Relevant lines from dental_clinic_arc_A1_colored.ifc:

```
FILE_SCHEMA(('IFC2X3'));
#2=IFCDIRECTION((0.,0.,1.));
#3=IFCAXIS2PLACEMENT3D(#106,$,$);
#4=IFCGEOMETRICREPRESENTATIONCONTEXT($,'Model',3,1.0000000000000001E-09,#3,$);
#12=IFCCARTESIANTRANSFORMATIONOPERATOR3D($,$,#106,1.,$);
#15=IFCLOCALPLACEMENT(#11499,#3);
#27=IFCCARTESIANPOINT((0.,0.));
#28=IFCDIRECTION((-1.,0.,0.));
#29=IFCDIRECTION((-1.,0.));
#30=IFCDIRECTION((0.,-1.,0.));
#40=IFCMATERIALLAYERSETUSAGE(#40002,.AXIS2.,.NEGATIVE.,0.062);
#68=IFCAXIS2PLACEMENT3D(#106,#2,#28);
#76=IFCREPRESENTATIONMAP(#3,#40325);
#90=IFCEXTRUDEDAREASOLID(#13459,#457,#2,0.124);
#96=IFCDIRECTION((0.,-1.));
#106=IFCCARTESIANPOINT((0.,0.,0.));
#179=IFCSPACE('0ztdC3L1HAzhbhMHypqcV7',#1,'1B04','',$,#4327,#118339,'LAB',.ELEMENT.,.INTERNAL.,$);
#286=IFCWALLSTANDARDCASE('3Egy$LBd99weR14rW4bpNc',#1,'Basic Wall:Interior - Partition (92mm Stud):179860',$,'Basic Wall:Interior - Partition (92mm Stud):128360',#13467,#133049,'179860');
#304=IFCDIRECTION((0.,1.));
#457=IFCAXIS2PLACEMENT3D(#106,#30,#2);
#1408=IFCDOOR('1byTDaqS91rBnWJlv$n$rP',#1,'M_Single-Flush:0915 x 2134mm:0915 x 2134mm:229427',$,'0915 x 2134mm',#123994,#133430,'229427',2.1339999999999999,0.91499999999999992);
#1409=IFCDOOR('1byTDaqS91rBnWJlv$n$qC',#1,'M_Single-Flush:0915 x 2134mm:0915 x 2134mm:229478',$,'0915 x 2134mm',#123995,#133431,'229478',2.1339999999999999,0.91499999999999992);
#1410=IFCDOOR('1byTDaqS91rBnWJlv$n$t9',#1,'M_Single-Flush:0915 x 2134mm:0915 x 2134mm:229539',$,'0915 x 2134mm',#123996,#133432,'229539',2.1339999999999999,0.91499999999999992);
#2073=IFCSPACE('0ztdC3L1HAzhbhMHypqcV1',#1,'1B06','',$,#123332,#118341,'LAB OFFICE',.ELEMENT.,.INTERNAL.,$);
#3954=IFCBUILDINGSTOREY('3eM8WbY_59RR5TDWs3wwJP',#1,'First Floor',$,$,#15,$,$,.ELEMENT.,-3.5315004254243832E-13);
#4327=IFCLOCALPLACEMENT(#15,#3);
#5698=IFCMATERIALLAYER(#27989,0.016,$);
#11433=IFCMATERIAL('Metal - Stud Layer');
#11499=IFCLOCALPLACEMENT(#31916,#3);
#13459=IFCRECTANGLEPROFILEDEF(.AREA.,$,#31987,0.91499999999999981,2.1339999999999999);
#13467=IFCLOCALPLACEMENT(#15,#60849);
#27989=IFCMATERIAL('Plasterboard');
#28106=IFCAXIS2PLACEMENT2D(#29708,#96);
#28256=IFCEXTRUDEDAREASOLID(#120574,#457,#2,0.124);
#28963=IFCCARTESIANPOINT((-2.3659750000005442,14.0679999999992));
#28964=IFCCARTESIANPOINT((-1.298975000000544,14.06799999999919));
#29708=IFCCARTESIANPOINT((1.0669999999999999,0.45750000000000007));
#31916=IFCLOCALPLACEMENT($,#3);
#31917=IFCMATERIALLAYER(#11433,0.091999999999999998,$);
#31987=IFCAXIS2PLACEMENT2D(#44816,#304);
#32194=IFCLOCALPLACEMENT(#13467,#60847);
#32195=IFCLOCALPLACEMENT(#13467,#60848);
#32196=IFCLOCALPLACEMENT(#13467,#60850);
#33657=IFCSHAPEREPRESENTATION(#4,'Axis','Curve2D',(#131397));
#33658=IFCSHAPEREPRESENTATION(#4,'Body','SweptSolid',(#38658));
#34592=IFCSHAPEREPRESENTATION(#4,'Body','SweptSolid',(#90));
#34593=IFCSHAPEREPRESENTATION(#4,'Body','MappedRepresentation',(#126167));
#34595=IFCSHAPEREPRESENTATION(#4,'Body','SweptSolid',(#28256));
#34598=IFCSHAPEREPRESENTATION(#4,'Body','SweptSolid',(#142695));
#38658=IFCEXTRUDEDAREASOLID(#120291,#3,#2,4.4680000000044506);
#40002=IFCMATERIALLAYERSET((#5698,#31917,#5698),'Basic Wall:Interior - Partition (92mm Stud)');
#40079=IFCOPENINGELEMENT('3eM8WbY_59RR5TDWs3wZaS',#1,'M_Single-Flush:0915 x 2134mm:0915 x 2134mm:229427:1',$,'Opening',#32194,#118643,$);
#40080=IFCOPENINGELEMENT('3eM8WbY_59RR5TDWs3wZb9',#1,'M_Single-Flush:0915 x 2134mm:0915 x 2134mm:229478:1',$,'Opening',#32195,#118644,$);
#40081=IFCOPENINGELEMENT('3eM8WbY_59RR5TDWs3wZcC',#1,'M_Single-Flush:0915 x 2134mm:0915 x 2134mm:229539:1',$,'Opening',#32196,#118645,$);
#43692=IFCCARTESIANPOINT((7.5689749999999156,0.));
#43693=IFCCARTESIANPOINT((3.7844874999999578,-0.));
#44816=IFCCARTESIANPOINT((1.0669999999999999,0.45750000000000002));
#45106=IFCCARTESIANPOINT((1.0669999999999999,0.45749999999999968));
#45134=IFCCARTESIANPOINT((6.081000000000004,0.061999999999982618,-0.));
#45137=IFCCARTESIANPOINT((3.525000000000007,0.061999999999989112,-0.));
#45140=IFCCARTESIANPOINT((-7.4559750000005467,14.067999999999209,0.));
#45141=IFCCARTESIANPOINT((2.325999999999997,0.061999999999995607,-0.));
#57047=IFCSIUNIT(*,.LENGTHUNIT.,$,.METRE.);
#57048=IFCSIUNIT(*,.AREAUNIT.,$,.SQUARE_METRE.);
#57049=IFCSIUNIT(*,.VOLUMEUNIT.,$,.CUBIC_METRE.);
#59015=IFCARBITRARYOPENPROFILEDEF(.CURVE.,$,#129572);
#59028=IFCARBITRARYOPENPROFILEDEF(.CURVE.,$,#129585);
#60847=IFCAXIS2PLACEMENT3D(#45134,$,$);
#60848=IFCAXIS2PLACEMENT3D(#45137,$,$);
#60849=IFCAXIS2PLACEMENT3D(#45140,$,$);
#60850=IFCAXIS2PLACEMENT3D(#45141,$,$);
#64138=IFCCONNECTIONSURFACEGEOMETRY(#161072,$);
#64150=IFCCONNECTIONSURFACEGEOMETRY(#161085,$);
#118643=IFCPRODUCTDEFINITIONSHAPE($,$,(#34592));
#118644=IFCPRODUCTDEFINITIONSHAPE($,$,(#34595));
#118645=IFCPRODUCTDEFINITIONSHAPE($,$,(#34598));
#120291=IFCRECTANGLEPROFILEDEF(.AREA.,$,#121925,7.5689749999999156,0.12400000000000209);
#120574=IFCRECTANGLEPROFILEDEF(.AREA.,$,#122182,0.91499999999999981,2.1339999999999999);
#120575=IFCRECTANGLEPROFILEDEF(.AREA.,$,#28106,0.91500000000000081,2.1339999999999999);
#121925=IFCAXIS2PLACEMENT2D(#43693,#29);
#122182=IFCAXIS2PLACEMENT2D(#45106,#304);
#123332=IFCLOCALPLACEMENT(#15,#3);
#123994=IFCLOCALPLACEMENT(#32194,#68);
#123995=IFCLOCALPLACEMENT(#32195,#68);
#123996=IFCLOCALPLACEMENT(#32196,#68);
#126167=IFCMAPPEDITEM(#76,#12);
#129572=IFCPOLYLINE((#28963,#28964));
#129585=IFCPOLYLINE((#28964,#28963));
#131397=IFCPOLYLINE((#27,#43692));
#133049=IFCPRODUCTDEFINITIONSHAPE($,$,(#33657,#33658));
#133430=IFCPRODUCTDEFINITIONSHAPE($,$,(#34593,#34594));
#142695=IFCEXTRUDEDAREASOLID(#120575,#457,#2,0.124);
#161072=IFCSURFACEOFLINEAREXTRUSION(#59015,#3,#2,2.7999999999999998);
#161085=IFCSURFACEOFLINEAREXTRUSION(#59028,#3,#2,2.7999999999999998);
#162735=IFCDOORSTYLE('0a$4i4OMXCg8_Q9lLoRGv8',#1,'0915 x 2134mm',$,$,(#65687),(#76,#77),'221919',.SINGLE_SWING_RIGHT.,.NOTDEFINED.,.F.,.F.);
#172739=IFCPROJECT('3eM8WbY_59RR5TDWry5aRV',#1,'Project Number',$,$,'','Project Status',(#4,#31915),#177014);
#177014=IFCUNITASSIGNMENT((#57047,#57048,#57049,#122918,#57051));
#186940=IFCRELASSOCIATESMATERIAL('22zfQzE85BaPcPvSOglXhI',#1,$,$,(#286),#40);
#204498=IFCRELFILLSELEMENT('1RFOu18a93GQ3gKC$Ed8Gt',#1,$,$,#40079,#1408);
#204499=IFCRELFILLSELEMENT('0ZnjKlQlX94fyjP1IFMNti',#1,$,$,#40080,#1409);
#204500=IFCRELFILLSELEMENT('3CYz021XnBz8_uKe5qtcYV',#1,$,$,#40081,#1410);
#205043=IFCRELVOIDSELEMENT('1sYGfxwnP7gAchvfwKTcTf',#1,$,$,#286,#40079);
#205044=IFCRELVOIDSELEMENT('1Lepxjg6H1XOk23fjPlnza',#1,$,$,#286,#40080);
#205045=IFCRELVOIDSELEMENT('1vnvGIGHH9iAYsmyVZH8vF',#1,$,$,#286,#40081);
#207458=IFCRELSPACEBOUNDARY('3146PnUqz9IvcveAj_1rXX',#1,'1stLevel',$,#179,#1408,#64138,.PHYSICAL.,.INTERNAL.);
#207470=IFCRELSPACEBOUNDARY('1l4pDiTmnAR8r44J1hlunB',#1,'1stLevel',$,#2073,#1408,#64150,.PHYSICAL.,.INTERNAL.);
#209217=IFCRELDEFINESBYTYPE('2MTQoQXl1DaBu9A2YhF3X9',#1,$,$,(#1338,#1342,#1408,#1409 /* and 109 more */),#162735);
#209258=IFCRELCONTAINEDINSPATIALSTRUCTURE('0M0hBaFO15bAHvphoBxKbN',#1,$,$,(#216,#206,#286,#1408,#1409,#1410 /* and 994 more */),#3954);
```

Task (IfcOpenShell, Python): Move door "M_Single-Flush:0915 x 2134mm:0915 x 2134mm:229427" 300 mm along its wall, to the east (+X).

```python
import numpy as np
import ifcopenshell
import ifcopenshell.api.geometry
import ifcopenshell.util.placement
import ifcopenshell.util.unit

model = ifcopenshell.open("dental_clinic_arc_A1_colored.ifc")
unit_scale = ifcopenshell.util.unit.calculate_unit_scale(model)

door = model.by_guid("1byTDaqS91rBnWJlv$n$rP")
opening = door.FillsVoids[0].RelatingOpeningElement
wall = opening.VoidsElements[0].RelatingBuildingElement

wall_matrix = ifcopenshell.util.placement.get_local_placement(wall.ObjectPlacement)
shift = wall_matrix[:3, 0] * 0.3 / unit_scale
before = ifcopenshell.util.placement.get_local_placement(door.ObjectPlacement)[:3, 3].copy()

# The door is placed relative to its opening, so it follows when the opening moves.
matrix = ifcopenshell.util.placement.get_local_placement(opening.ObjectPlacement)
matrix[:3, 3] += shift
ifcopenshell.api.geometry.edit_object_placement(
    model, product=opening, matrix=matrix, is_si=False, should_transform_children=True
)

# Space boundary surfaces are stored in each space's coordinates; move them too.
for rel in door.ProvidesBoundaries:
    if not rel.ConnectionGeometry:
        continue
    surface = rel.ConnectionGeometry.SurfaceOnRelatingElement
    space_matrix = ifcopenshell.util.placement.get_local_placement(rel.RelatingSpace.ObjectPlacement)
    point = np.array(surface.Position.Location.Coordinates) + space_matrix[:3, :3].T @ shift
    surface.Position = model.createIfcAxis2Placement3D(
        model.createIfcCartesianPoint(point.tolist()), surface.Position.Axis, surface.Position.RefDirection
    )

after = ifcopenshell.util.placement.get_local_placement(door.ObjectPlacement)[:3, 3]
print("door moved by", (after - before).round(3) + 0.0)

model.write("dental_clinic_arc_A1_colored_v2.ifc")
```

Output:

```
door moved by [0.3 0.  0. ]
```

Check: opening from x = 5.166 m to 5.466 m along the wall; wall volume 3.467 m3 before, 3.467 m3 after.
